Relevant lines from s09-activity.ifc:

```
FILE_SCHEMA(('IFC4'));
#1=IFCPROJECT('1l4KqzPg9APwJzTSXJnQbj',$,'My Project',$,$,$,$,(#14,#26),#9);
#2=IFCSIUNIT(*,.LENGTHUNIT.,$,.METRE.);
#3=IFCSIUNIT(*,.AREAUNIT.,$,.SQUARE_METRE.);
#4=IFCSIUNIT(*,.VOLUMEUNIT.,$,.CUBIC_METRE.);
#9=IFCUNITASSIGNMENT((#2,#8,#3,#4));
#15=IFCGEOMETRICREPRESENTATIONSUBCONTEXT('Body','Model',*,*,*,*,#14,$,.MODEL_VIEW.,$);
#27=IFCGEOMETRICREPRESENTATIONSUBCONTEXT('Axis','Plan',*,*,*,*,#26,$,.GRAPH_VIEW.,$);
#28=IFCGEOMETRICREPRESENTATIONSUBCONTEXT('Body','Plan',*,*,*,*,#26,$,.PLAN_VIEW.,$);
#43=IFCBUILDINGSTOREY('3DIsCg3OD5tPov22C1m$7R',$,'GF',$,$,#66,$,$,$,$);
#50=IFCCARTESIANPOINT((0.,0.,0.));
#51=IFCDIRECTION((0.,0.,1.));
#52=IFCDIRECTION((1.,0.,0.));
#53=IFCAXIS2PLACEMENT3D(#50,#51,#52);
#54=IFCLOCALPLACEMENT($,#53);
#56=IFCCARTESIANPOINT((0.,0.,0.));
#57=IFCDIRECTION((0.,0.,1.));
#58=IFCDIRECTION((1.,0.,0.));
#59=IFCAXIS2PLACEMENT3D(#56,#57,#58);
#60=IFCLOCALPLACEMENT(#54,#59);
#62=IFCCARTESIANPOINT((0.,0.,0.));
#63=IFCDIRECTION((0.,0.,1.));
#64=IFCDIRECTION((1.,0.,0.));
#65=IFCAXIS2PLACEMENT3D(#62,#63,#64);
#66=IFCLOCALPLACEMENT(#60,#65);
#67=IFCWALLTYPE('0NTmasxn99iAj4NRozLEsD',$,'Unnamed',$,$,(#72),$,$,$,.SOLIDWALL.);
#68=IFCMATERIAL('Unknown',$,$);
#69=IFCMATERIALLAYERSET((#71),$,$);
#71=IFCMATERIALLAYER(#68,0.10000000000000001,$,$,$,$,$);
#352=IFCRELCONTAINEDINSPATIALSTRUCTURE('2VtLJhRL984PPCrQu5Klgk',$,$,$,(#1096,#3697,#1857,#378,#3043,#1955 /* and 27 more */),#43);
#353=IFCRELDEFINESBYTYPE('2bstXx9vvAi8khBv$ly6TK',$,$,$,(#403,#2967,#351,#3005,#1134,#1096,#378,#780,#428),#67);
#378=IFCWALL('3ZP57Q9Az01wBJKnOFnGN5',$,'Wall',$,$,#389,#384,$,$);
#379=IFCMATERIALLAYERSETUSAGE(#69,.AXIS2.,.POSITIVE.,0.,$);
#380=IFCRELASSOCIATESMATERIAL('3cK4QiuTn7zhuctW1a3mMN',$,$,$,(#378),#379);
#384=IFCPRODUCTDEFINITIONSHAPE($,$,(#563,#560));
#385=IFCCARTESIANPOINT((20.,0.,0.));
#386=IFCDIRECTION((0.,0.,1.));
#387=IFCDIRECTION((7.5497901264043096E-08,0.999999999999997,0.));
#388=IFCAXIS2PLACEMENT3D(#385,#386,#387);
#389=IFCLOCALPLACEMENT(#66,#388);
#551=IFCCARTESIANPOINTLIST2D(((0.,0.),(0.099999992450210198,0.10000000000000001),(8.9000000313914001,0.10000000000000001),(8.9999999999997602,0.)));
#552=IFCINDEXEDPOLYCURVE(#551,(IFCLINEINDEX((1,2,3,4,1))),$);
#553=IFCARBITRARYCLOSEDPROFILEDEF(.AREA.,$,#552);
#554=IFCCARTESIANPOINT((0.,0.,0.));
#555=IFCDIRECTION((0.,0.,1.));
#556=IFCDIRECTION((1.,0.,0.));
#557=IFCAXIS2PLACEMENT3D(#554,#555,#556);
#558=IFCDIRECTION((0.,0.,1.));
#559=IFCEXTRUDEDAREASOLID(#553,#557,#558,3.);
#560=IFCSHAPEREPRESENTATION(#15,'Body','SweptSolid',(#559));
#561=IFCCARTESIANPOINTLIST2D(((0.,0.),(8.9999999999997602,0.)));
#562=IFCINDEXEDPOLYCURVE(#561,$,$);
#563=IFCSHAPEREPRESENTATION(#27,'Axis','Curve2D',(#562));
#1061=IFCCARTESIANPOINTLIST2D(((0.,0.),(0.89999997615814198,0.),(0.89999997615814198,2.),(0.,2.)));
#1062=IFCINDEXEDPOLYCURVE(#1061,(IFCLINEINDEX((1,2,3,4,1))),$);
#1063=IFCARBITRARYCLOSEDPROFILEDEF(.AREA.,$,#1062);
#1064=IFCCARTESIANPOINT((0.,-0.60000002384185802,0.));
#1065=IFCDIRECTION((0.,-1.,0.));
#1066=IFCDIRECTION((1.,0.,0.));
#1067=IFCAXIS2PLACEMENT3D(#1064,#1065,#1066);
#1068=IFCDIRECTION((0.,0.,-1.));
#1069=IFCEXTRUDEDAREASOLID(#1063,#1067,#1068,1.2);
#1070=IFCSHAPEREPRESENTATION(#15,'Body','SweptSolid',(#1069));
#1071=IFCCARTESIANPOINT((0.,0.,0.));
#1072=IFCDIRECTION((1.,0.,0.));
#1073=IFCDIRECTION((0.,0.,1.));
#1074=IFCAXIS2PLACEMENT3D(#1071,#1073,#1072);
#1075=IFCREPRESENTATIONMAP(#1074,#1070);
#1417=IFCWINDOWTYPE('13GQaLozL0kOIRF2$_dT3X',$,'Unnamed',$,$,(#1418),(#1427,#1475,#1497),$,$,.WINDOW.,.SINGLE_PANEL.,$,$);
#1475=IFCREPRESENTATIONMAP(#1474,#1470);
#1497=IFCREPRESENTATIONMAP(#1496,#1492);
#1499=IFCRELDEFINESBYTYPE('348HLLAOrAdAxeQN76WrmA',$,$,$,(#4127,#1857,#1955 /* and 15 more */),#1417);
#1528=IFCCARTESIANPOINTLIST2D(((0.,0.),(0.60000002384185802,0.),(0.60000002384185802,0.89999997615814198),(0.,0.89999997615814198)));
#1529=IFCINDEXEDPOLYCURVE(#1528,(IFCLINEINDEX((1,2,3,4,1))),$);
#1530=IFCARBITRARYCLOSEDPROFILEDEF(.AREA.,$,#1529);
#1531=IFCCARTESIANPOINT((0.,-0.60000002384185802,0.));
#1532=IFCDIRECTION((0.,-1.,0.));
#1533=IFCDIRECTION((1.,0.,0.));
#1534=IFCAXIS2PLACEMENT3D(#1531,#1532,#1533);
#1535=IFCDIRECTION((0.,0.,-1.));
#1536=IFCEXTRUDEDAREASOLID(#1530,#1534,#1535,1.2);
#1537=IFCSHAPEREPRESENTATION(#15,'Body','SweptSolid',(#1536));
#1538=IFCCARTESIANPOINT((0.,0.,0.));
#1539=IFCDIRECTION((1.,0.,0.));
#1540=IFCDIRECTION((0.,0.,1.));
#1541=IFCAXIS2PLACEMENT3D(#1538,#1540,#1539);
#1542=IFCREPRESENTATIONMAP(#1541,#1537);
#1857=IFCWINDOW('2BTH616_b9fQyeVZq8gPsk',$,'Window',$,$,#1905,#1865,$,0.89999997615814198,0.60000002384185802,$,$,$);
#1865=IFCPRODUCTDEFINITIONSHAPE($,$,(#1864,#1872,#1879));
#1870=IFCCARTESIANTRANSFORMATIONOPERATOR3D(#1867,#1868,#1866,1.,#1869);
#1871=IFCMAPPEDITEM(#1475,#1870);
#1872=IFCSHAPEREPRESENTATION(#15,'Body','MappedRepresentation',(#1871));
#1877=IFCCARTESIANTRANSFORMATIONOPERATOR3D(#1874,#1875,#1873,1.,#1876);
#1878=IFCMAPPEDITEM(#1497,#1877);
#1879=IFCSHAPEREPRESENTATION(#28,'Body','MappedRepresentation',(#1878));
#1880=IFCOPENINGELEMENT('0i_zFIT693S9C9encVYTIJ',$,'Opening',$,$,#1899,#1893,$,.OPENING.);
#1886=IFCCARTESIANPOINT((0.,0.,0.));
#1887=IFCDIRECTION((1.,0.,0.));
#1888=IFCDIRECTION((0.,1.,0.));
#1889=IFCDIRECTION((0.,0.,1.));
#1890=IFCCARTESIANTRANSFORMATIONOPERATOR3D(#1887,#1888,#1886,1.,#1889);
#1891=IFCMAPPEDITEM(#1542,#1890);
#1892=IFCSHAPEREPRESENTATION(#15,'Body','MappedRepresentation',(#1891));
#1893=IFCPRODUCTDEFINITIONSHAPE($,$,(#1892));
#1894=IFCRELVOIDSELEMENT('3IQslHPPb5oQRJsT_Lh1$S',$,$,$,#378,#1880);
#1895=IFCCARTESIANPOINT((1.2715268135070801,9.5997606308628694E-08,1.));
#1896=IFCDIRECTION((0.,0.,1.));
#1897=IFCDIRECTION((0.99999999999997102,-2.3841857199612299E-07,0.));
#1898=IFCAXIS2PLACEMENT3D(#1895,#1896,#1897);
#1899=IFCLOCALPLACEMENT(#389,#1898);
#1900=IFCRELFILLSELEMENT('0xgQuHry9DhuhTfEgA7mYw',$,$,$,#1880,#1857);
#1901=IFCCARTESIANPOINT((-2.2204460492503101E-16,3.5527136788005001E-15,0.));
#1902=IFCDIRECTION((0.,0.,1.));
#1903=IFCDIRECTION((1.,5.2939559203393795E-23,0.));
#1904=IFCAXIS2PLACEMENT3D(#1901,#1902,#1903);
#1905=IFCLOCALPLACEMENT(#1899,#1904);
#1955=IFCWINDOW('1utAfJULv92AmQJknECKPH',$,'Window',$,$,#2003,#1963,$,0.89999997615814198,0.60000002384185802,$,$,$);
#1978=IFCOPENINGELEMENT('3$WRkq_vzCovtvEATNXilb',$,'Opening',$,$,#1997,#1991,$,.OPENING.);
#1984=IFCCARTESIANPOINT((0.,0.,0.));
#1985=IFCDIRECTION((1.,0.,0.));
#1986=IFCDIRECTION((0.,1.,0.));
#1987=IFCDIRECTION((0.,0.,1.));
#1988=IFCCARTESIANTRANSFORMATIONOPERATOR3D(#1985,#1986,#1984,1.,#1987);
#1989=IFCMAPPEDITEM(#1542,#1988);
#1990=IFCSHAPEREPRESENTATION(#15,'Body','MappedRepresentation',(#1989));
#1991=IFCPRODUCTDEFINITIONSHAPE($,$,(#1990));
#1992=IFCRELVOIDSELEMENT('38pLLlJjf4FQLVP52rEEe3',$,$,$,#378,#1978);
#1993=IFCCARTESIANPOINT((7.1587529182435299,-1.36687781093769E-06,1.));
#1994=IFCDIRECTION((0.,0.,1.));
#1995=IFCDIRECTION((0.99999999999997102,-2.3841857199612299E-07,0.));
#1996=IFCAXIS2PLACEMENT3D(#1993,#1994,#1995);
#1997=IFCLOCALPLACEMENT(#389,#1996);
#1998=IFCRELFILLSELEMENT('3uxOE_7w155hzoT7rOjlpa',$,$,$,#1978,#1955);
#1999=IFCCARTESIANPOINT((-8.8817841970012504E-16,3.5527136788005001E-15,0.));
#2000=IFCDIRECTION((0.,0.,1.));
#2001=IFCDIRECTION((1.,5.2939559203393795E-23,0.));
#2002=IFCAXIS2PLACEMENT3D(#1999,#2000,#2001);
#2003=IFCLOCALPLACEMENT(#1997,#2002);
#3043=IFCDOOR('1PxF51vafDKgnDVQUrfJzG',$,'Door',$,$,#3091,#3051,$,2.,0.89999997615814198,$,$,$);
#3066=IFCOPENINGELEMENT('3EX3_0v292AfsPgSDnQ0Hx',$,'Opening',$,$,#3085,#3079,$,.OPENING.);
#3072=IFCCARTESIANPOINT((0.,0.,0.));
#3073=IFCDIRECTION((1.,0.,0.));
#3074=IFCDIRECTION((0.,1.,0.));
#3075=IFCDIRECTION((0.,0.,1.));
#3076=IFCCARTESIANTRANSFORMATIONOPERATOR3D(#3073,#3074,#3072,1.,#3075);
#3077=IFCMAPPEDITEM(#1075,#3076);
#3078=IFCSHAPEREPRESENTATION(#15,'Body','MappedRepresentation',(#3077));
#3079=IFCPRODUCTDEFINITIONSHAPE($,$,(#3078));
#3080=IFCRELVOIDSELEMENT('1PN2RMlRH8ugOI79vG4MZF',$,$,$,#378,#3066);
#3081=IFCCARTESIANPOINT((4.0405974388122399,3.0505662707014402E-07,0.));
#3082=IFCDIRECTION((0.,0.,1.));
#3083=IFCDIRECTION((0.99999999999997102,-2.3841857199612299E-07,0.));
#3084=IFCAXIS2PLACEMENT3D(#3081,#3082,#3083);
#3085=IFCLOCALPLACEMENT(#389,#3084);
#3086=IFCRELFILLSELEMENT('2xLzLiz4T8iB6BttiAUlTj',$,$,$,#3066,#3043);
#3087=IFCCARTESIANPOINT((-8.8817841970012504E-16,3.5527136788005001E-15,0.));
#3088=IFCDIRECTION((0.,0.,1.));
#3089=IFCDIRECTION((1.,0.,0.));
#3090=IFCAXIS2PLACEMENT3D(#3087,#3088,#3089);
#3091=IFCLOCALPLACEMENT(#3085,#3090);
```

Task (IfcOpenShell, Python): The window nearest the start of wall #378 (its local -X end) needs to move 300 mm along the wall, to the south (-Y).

```python
import ifcopenshell
import ifcopenshell.api.geometry
import ifcopenshell.util.placement

model = ifcopenshell.open("s09-activity.ifc")

window = model.by_guid("2BTH616_b9fQyeVZq8gPsk")
opening = window.FillsVoids[0].RelatingOpeningElement
wall = opening.VoidsElements[0].RelatingBuildingElement

wall_matrix = ifcopenshell.util.placement.get_local_placement(wall.ObjectPlacement)
shift = wall_matrix[:3, 0] * -0.3
before = ifcopenshell.util.placement.get_local_placement(window.ObjectPlacement)[:3, 3].copy()

# The window is placed relative to its opening, so it follows when the opening moves.
matrix = ifcopenshell.util.placement.get_local_placement(opening.ObjectPlacement)
matrix[:3, 3] += shift
ifcopenshell.api.geometry.edit_object_placement(
    model, product=opening, matrix=matrix, is_si=False, should_transform_children=True
)

after = ifcopenshell.util.placement.get_local_placement(window.ObjectPlacement)[:3, 3]
print("window moved by", (after - before).round(3) + 0.0)

model.write("s09-activity-out.ifc")
```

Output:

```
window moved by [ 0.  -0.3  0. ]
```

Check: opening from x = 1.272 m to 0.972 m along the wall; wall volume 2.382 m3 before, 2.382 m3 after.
